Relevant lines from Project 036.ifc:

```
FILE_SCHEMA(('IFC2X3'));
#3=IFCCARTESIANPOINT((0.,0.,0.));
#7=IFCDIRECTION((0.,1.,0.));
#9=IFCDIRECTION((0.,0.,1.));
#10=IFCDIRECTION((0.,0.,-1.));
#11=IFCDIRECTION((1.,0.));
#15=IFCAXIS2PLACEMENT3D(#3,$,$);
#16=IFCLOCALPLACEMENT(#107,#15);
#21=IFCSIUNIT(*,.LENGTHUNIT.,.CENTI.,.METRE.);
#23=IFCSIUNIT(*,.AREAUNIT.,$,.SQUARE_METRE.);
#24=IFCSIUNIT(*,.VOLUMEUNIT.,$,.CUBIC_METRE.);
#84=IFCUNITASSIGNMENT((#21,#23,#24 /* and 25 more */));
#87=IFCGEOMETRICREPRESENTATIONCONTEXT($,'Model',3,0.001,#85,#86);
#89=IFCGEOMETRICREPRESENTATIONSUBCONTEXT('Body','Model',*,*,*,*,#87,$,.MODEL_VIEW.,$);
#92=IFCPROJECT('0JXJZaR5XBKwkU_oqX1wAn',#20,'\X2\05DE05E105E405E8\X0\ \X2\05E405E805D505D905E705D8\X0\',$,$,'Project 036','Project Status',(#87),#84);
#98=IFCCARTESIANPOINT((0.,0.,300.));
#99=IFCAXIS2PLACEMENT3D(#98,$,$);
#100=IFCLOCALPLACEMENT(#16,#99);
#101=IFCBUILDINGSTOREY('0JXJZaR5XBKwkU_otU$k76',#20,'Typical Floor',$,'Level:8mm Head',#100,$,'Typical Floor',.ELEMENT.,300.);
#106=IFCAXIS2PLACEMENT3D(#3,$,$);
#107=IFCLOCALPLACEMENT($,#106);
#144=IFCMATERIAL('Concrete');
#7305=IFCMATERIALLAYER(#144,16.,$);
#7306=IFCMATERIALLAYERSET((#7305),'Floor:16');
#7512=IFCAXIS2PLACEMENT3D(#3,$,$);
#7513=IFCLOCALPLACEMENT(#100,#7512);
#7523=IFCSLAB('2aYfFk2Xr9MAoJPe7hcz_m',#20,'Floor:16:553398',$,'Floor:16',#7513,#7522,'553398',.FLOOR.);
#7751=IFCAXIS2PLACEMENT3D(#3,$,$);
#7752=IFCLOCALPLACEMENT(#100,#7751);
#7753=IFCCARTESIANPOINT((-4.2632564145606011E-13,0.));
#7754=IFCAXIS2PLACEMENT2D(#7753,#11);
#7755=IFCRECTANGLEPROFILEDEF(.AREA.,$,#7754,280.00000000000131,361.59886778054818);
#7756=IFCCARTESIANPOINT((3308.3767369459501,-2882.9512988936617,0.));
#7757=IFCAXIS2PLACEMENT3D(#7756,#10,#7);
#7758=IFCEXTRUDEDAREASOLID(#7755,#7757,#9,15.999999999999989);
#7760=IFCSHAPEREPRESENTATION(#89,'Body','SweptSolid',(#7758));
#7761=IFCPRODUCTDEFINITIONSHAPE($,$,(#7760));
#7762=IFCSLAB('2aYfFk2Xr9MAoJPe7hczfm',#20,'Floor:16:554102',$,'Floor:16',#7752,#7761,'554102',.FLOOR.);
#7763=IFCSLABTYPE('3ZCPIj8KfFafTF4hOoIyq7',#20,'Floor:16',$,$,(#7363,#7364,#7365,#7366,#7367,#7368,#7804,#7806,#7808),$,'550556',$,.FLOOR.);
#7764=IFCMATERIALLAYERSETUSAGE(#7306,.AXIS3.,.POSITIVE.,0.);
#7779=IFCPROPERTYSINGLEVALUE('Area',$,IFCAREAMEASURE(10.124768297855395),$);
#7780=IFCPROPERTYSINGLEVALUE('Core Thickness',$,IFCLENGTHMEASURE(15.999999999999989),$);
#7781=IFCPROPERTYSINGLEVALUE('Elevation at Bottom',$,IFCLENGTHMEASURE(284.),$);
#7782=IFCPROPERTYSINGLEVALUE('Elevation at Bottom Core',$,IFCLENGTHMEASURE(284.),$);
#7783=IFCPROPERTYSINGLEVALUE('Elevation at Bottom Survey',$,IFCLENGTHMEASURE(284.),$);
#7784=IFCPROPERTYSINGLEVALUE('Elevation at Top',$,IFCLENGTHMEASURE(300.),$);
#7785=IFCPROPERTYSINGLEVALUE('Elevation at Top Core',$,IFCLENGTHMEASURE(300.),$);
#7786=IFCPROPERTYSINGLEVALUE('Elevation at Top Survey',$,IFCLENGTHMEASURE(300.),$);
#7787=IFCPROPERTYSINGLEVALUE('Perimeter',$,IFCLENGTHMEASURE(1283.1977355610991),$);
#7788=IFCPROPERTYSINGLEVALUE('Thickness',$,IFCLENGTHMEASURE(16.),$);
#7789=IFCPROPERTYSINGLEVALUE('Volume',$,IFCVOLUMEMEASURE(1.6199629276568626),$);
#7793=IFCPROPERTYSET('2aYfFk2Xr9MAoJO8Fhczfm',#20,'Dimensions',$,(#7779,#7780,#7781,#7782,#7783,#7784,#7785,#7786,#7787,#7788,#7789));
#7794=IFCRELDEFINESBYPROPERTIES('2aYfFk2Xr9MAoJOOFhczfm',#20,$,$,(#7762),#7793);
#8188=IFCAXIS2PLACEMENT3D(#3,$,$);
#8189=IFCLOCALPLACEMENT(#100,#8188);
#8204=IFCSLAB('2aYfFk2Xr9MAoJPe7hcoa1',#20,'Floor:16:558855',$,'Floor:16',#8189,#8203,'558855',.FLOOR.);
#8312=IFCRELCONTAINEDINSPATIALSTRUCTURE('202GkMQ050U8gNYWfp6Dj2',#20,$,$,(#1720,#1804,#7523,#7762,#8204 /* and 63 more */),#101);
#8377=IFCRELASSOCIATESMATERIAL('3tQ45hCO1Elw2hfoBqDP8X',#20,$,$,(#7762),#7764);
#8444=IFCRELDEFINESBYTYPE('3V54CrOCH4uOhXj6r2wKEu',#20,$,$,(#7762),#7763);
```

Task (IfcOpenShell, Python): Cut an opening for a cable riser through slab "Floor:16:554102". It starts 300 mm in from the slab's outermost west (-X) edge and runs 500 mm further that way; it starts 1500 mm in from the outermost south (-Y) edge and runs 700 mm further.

```python
import numpy as np
import ifcopenshell
import ifcopenshell.api.feature
import ifcopenshell.api.geometry
import ifcopenshell.api.pset
import ifcopenshell.api.root
import ifcopenshell.geom
import ifcopenshell.util.element
import ifcopenshell.util.placement
import ifcopenshell.util.representation
import ifcopenshell.util.shape
import ifcopenshell.util.unit

model = ifcopenshell.open("Project 036.ifc")
unit_scale = ifcopenshell.util.unit.calculate_unit_scale(model)
area_scale = ifcopenshell.util.unit.calculate_unit_scale(model, "AREAUNIT")
volume_scale = ifcopenshell.util.unit.calculate_unit_scale(model, "VOLUMEUNIT")
settings = ifcopenshell.geom.settings()


def volume(element):
    """Net volume in cubic metres, openings subtracted."""
    shape = ifcopenshell.geom.create_shape(settings, element)
    return ifcopenshell.util.shape.get_volume(shape.geometry)


slab = model.by_guid("2aYfFk2Xr9MAoJPe7hczfm")
before = volume(slab)

# Extent in the slab's own axes, in metres. The edges named are its -X and -Y sides.
slab_shape = ifcopenshell.geom.create_shape(settings, slab)
vertices = ifcopenshell.util.shape.get_vertices(slab_shape.geometry)
x_min, y_min, bottom = vertices.min(axis=0)
top = vertices[:, 2].max()

opening = ifcopenshell.api.root.create_entity(model, ifc_class="IfcOpeningElement", name="Cable riser opening")
context = ifcopenshell.util.representation.get_context(model, "Model", "Body", "MODEL_VIEW")
width, depth = 0.5, 0.7
outline = [(0.0, 0.0), (width, 0.0), (width, depth), (0.0, depth), (0.0, 0.0)]
# Overshoot both faces by 50 mm so the cut is clean.
shape = ifcopenshell.api.geometry.add_slab_representation(
    model, context=context, depth=top - bottom + 0.1, polyline=outline
)
ifcopenshell.api.geometry.assign_representation(model, product=opening, representation=shape)

matrix = ifcopenshell.util.placement.get_local_placement(slab.ObjectPlacement)
matrix[:, 3] = matrix @ np.append(np.array([x_min + 0.3, y_min + 1.5, bottom - 0.05]) / unit_scale, 1.0)
ifcopenshell.api.geometry.edit_object_placement(model, product=opening, matrix=matrix, is_si=False)
ifcopenshell.api.feature.add_feature(model, feature=opening, element=slab)

after = volume(slab)

# Update the slab's stored quantities.
pset = model.by_id(ifcopenshell.util.element.get_pset(slab, "Dimensions", should_inherit=False)["id"])
ifcopenshell.api.pset.edit_pset(model, pset=pset, properties={
    "Area": model.create_entity("IfcAreaMeasure", after / (top - bottom) / area_scale),
    "Volume": model.create_entity("IfcVolumeMeasure", after / volume_scale),
})

print(f"slab volume {before:.3f} -> {after:.3f} m3")

model.write("Project 036_rev.ifc")
```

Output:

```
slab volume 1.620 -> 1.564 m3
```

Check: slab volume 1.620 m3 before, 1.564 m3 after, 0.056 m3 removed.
